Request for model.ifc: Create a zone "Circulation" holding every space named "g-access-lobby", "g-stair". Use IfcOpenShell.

First a look at what the model holds.

```python
import ifcopenshell

model = ifcopenshell.open("model.ifc")
print(model.schema)
seen = {}
for space in model.by_type("IfcSpace"):
    seen[space.LongName] = seen.get(space.LongName, 0) + 1
for name, count in sorted(seen.items(), key=str):
    print(count, "x", name)
print("zones:", [z.Name for z in model.by_type("IfcZone")][:20])
```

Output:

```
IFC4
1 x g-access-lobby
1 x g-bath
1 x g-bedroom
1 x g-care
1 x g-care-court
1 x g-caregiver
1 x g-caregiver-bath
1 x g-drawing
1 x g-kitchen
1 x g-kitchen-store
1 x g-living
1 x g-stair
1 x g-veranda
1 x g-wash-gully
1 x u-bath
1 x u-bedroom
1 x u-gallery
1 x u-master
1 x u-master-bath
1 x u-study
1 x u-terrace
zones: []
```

```python
import ifcopenshell
import ifcopenshell.api.group
import ifcopenshell.api.root

model = ifcopenshell.open("model.ifc")

names = {"g-access-lobby", "g-stair"}
spaces = [s for s in model.by_type("IfcSpace") if s.LongName in names]

zone = ifcopenshell.api.root.create_entity(model, ifc_class="IfcZone", name="Circulation")
ifcopenshell.api.group.assign_group(model, products=spaces, group=zone)
print(len(spaces), "spaces in", zone.Name)

model.write("model_updated.ifc")
```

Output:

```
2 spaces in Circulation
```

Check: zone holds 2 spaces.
